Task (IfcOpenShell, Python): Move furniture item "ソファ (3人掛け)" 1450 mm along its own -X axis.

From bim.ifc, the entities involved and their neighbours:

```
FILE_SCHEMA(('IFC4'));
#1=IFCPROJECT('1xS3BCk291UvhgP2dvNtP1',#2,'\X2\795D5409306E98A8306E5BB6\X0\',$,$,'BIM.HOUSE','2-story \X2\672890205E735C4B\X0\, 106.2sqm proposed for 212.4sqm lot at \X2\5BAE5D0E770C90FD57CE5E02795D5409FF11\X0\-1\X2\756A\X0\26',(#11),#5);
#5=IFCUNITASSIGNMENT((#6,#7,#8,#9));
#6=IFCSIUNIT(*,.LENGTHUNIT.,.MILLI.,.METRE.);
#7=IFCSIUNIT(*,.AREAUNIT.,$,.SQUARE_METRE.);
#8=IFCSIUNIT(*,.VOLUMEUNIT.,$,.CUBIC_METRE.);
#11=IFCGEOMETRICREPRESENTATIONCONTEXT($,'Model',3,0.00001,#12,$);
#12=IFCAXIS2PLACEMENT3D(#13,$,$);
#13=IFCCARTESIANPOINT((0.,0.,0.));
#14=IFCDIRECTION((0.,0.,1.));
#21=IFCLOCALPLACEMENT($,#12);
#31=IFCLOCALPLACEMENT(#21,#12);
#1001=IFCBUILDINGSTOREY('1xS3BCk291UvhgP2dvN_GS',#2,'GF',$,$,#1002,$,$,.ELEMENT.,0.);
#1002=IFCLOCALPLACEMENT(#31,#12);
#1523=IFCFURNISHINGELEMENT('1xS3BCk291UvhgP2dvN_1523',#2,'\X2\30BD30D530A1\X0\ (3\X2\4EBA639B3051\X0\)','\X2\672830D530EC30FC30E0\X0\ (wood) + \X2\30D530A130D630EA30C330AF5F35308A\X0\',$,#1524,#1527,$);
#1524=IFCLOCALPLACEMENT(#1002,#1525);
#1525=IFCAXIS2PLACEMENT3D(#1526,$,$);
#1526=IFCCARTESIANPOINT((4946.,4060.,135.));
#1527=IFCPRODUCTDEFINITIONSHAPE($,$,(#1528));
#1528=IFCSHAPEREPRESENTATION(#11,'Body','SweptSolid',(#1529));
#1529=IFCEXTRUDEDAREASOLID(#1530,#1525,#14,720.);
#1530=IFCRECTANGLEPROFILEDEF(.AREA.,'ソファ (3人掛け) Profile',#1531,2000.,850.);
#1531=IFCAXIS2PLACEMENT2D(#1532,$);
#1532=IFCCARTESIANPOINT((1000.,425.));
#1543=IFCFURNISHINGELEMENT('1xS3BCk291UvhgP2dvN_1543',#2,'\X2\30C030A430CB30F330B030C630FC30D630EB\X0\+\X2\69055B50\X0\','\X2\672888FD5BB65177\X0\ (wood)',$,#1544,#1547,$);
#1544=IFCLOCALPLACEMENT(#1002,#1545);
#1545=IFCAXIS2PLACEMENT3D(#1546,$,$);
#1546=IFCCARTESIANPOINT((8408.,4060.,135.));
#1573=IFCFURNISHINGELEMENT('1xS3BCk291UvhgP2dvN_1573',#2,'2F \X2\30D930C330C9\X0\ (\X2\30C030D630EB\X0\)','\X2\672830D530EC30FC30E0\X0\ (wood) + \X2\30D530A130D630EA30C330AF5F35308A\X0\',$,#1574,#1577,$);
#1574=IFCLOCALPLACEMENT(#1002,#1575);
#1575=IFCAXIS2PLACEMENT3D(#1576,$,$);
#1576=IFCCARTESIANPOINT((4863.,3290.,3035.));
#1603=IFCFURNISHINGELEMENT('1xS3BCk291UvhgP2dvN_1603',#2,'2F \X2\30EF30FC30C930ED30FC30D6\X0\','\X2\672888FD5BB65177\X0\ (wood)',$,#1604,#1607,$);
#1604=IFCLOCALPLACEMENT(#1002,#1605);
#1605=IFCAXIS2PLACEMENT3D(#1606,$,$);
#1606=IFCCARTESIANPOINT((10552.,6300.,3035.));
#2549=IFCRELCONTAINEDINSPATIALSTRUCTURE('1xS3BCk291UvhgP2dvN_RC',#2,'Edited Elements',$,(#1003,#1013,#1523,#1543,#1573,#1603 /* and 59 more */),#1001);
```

```python
import ifcopenshell
import ifcopenshell.api.geometry
import ifcopenshell.util.placement

model = ifcopenshell.open("bim.ifc")

item = model.by_guid("1xS3BCk291UvhgP2dvN_1523")
matrix = ifcopenshell.util.placement.get_local_placement(item.ObjectPlacement)
matrix[:3, 3] -= matrix[:3, 0] * 1450.0
ifcopenshell.api.geometry.edit_object_placement(model, product=item, matrix=matrix, is_si=False)

print(ifcopenshell.util.placement.get_local_placement(item.ObjectPlacement).round(3) + 0.0)

model.write("bim_edited.ifc")
```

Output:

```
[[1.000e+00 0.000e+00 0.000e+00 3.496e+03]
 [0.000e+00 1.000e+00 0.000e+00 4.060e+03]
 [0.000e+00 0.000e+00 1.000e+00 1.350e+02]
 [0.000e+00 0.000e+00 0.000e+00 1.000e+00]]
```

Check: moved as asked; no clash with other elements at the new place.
